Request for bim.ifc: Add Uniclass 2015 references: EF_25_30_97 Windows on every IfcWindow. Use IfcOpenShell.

First a look at what the model holds.

```python
import ifcopenshell

model = ifcopenshell.open("bim.ifc")
print(model.schema)
print("classifications:", [c.Name for c in model.by_type("IfcClassification")])
for ifc_class in ("IfcDoor", "IfcRoof", "IfcStair", "IfcWall", "IfcWindow"):
    print(ifc_class, len(model.by_type(ifc_class)))
```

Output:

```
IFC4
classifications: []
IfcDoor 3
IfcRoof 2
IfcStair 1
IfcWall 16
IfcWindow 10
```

```python
import ifcopenshell
import ifcopenshell.api.classification

model = ifcopenshell.open("bim.ifc")

system = ifcopenshell.api.classification.add_classification(model, classification="Uniclass 2015")

codes = {
    "IfcWindow": ("EF_25_30_97", "Windows"),
}
for ifc_class, (code, name) in codes.items():
    products = model.by_type(ifc_class)
    ifcopenshell.api.classification.add_reference(
        model, products=products, classification=system, identification=code, name=name
    )
    print(code, len(products))

model.write("bim_v2.ifc")
```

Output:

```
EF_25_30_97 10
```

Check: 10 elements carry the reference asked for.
